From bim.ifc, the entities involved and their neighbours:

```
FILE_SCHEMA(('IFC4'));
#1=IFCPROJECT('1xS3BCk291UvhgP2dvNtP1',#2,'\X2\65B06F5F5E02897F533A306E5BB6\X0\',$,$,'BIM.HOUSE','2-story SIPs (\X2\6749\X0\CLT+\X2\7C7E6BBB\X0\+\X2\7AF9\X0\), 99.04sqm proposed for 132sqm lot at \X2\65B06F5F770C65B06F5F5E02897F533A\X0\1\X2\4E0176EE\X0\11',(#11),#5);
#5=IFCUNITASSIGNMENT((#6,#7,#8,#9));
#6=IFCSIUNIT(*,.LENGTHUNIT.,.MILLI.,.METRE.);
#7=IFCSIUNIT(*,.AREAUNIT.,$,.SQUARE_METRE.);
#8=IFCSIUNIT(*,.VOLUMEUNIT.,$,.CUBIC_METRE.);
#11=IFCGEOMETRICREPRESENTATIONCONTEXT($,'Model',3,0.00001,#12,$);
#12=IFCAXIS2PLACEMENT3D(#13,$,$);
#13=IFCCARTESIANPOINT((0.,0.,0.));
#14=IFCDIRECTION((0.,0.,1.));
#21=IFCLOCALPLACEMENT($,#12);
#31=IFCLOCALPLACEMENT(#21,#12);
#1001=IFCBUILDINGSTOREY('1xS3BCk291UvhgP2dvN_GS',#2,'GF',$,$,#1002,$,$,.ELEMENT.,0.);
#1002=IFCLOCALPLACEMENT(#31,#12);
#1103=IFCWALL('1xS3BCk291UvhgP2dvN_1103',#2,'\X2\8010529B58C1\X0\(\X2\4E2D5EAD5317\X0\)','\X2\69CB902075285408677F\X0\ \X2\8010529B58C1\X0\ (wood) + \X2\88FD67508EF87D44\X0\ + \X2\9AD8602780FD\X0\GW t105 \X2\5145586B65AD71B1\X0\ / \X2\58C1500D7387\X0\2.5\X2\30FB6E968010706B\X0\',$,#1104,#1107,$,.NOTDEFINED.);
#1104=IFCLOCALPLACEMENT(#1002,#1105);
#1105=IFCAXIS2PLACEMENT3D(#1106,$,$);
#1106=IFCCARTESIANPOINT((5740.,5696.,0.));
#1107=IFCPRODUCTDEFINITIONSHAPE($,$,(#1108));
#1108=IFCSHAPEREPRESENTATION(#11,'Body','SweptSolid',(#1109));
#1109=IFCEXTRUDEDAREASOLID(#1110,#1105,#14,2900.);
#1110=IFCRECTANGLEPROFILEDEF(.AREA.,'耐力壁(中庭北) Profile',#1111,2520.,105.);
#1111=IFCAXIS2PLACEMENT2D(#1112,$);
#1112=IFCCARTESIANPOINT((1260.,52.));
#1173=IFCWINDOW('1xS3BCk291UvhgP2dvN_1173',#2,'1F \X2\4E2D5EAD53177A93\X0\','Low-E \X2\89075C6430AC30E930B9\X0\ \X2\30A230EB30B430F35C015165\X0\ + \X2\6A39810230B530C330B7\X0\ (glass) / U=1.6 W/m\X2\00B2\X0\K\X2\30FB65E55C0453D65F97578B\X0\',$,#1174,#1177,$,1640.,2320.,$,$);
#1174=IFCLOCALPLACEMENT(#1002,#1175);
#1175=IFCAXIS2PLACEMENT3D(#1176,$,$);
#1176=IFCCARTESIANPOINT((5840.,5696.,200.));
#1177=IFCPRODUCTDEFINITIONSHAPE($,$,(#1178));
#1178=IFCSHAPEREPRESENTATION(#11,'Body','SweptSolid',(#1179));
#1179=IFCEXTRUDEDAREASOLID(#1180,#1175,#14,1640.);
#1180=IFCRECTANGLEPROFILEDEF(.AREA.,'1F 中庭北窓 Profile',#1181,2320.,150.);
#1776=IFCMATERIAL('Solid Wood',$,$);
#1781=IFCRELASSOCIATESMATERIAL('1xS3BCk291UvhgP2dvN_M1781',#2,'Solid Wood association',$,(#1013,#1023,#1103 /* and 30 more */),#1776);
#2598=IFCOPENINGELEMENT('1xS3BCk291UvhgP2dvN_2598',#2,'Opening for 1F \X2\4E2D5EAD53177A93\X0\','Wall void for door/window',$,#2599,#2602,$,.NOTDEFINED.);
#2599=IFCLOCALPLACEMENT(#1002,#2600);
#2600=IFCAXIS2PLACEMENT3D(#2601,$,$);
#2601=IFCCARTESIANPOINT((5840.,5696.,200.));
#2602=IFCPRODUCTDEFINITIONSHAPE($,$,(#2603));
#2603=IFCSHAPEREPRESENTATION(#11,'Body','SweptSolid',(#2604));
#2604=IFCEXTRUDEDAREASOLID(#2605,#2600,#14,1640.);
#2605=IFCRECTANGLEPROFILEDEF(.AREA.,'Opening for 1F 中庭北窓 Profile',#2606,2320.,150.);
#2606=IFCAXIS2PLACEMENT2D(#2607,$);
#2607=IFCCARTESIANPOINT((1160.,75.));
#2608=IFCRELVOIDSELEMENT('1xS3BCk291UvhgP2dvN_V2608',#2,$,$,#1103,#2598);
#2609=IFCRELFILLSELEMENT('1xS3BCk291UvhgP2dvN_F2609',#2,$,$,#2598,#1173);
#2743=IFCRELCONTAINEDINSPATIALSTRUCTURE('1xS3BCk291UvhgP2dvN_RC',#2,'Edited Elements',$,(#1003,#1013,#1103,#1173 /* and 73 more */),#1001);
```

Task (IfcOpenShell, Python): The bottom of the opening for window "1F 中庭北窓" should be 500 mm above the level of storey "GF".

```python
import numpy as np
import ifcopenshell
import ifcopenshell.api.geometry
import ifcopenshell.geom
import ifcopenshell.util.element
import ifcopenshell.util.placement
import ifcopenshell.util.shape
import ifcopenshell.util.unit

model = ifcopenshell.open("bim.ifc")
unit_scale = ifcopenshell.util.unit.calculate_unit_scale(model)

window = model.by_guid("1xS3BCk291UvhgP2dvN_1173")
opening = window.FillsVoids[0].RelatingOpeningElement
storey = ifcopenshell.util.element.get_container(window, ifc_class="IfcBuildingStorey")
level = ifcopenshell.util.placement.get_local_placement(storey.ObjectPlacement)[2, 3]

# The opening's origin need not be at the sill, so measure its lowest point.
shape = ifcopenshell.geom.create_shape(ifcopenshell.geom.settings(), opening)
bottom = ifcopenshell.util.shape.get_shape_bottom_elevation(shape, shape.geometry) / unit_scale
dz = level + 0.5 / unit_scale - bottom

shift = np.array([0.0, 0.0, dz])
# The window is not placed relative to its opening, so move both.
for product in (opening, window):
    matrix = ifcopenshell.util.placement.get_local_placement(product.ObjectPlacement)
    matrix[:3, 3] += shift
    ifcopenshell.api.geometry.edit_object_placement(model, product=product, matrix=matrix, is_si=False)

print(f"moved by {dz * unit_scale:+.3f} m")

model.write("bim_updated.ifc")
```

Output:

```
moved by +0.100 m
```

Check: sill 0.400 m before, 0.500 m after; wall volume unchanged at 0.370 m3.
